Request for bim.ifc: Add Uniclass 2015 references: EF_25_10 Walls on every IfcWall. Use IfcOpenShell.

First a look at what the model holds.

```python
import ifcopenshell

model = ifcopenshell.open("bim.ifc")
print(model.schema)
print("classifications:", [c.Name for c in model.by_type("IfcClassification")])
for ifc_class in ("IfcDoor", "IfcRoof", "IfcStair", "IfcWall", "IfcWindow"):
    print(ifc_class, len(model.by_type(ifc_class)))
```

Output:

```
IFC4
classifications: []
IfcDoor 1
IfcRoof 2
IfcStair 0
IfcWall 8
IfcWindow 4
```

```python
import ifcopenshell
import ifcopenshell.api.classification

model = ifcopenshell.open("bim.ifc")

system = ifcopenshell.api.classification.add_classification(model, classification="Uniclass 2015")

codes = {
    "IfcWall": ("EF_25_10", "Walls"),
}
for ifc_class, (code, name) in codes.items():
    products = model.by_type(ifc_class)
    ifcopenshell.api.classification.add_reference(
        model, products=products, classification=system, identification=code, name=name
    )
    print(code, len(products))

model.write("bim_rev.ifc")
```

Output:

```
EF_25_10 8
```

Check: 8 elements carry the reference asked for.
